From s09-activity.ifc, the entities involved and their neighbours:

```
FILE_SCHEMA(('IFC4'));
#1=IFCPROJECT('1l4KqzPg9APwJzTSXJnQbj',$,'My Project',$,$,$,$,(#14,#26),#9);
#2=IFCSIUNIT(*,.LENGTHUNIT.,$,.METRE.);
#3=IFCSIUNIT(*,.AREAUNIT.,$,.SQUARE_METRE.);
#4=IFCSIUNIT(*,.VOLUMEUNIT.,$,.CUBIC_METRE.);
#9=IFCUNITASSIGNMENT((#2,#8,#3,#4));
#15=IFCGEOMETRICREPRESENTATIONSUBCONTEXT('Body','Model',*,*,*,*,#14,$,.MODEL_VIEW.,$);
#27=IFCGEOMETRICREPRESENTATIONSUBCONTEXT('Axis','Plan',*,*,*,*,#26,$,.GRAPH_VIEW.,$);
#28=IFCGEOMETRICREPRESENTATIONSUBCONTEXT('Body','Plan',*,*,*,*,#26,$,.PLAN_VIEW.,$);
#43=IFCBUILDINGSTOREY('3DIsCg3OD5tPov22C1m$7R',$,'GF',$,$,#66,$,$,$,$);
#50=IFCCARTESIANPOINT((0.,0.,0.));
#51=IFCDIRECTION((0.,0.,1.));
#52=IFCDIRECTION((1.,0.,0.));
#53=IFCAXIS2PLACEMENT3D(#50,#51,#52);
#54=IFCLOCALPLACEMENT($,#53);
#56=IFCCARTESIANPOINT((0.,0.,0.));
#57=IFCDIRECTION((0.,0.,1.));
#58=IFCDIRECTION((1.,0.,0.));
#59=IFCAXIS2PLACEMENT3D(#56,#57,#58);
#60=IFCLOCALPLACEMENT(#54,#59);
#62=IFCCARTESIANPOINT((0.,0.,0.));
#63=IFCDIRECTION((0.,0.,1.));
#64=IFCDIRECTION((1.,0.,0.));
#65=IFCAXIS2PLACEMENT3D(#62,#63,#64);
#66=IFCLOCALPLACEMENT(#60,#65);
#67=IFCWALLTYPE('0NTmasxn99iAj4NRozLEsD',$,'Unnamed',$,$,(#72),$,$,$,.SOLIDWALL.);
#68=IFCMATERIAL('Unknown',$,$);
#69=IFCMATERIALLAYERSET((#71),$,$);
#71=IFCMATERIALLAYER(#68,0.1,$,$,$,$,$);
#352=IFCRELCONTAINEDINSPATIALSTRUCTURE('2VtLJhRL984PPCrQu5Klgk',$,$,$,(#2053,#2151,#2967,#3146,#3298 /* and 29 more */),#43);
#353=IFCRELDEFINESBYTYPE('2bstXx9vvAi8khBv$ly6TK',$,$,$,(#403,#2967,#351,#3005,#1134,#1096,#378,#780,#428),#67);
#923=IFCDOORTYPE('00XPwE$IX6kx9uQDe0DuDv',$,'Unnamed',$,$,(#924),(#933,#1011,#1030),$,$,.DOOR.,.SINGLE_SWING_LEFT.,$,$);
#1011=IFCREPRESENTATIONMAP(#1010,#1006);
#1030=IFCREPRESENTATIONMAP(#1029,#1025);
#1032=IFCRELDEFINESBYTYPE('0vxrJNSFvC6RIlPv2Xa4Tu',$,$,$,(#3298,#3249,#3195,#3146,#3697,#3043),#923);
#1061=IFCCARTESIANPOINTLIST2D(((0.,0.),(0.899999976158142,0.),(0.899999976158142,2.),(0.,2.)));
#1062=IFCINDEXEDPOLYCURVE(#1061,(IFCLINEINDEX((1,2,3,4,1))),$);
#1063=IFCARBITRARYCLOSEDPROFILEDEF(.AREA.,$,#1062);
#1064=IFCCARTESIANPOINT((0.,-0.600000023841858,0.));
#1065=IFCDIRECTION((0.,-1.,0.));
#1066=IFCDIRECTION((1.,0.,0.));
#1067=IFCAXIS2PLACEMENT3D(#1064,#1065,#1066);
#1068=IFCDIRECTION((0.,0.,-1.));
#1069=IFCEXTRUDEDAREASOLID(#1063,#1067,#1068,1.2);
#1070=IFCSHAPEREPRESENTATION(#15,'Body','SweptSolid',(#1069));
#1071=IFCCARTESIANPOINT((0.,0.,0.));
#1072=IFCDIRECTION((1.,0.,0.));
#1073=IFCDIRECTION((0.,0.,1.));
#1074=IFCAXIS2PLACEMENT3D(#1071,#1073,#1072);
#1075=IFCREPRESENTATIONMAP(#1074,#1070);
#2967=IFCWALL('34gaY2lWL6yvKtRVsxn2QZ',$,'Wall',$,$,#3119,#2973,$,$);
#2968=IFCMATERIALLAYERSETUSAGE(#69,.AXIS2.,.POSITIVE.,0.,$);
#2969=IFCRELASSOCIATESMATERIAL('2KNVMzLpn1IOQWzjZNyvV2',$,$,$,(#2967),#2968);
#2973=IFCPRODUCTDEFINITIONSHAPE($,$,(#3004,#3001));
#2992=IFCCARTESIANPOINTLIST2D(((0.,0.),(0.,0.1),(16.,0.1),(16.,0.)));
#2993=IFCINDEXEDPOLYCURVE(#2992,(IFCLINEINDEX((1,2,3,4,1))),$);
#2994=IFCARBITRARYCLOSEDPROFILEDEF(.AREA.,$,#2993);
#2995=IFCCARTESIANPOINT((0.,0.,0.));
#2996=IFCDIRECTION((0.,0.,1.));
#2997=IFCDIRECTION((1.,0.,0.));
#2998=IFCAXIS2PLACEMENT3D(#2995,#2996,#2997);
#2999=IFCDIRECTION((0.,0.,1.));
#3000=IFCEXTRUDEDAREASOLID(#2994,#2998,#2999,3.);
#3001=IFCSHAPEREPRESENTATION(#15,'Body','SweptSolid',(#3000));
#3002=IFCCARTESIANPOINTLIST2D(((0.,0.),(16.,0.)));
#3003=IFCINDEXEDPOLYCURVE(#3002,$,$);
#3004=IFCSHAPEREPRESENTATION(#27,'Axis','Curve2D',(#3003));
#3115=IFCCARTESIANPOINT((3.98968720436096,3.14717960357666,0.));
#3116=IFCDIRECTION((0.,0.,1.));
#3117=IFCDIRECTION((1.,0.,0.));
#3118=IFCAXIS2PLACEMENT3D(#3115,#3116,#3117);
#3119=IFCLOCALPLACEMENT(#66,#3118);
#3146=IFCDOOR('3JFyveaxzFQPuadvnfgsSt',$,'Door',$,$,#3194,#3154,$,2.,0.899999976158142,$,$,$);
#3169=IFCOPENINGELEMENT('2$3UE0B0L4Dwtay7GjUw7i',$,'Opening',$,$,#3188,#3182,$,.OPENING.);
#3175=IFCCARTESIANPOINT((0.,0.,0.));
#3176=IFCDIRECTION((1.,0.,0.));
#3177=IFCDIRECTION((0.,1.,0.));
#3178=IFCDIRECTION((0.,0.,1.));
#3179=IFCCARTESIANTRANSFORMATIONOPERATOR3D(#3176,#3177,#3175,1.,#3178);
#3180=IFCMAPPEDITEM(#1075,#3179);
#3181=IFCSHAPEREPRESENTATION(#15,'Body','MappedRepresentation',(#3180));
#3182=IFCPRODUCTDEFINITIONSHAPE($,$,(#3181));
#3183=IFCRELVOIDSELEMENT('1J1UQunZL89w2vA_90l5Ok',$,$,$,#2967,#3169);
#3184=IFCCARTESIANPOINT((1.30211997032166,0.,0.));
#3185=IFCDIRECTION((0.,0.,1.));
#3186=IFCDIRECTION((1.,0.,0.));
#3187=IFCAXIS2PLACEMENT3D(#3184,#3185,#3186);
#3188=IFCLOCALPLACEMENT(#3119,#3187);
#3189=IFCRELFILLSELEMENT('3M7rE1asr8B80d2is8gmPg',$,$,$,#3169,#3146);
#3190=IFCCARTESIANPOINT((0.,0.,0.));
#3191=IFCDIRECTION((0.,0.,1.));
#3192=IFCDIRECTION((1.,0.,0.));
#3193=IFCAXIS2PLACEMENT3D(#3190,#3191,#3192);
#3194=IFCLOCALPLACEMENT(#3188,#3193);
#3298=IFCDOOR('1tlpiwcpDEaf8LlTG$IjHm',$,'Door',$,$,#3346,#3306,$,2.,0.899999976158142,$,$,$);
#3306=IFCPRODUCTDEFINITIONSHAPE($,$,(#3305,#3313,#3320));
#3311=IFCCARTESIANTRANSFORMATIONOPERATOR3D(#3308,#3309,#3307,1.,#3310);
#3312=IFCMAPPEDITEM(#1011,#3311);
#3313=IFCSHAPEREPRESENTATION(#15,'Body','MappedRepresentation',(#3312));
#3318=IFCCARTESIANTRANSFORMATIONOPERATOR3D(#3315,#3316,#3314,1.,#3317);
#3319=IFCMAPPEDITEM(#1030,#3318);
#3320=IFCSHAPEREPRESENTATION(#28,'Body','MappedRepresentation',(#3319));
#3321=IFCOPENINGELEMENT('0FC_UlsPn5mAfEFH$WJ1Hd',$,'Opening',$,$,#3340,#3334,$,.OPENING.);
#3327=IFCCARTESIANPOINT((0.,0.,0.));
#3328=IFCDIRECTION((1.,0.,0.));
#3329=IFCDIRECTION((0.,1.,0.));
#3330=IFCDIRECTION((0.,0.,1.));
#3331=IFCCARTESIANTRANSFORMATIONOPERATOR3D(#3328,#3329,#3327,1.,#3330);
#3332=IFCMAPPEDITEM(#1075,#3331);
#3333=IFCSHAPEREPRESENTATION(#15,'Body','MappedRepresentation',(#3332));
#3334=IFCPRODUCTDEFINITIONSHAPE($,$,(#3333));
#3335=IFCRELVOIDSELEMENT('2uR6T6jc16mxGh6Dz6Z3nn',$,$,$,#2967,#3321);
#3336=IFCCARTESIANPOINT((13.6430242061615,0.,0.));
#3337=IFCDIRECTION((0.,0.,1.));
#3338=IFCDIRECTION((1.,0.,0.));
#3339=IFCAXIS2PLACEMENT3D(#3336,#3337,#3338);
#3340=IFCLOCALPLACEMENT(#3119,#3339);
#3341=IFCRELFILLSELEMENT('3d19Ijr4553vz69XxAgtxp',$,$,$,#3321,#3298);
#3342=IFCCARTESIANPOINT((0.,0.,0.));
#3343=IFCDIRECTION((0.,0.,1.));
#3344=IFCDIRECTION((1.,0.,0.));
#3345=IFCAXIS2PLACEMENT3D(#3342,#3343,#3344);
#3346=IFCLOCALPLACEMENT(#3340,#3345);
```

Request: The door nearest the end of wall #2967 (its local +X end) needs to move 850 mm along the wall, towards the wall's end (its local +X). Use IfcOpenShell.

```python
import ifcopenshell
import ifcopenshell.api.geometry
import ifcopenshell.util.placement

model = ifcopenshell.open("s09-activity.ifc")

door = model.by_id(3298)
opening = door.FillsVoids[0].RelatingOpeningElement
wall = opening.VoidsElements[0].RelatingBuildingElement

wall_matrix = ifcopenshell.util.placement.get_local_placement(wall.ObjectPlacement)
shift = wall_matrix[:3, 0] * 0.85
before = ifcopenshell.util.placement.get_local_placement(door.ObjectPlacement)[:3, 3].copy()

# The door is placed relative to its opening, so it follows when the opening moves.
matrix = ifcopenshell.util.placement.get_local_placement(opening.ObjectPlacement)
matrix[:3, 3] += shift
ifcopenshell.api.geometry.edit_object_placement(
    model, product=opening, matrix=matrix, is_si=False, should_transform_children=True
)

after = ifcopenshell.util.placement.get_local_placement(door.ObjectPlacement)[:3, 3]
print("door moved by", (after - before).round(3) + 0.0)

model.write("s09-activity-out.ifc")
```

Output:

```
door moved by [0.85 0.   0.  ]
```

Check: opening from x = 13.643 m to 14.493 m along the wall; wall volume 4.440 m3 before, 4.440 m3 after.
